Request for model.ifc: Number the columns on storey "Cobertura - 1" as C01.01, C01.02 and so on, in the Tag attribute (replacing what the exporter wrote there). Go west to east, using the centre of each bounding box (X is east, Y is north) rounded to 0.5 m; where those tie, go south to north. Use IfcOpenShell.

First a look at what the model holds.

```python
import ifcopenshell
import ifcopenshell.util.element
import ifcopenshell.util.placement

model = ifcopenshell.open("model.ifc")
print(model.schema)
storey = next(s for s in model.by_type("IfcBuildingStorey") if s.Name == "Cobertura - 1")
columns = [e for e in ifcopenshell.util.element.get_decomposition(storey) if e.is_a("IfcColumn")]
for e in sorted(columns, key=lambda e: e.id()):
    origin = ifcopenshell.util.placement.get_local_placement(e.ObjectPlacement)[:3, 3]
    print(e.id(), e.Tag, e.Name, origin.round(2) + 0.0, sep=" | ")
```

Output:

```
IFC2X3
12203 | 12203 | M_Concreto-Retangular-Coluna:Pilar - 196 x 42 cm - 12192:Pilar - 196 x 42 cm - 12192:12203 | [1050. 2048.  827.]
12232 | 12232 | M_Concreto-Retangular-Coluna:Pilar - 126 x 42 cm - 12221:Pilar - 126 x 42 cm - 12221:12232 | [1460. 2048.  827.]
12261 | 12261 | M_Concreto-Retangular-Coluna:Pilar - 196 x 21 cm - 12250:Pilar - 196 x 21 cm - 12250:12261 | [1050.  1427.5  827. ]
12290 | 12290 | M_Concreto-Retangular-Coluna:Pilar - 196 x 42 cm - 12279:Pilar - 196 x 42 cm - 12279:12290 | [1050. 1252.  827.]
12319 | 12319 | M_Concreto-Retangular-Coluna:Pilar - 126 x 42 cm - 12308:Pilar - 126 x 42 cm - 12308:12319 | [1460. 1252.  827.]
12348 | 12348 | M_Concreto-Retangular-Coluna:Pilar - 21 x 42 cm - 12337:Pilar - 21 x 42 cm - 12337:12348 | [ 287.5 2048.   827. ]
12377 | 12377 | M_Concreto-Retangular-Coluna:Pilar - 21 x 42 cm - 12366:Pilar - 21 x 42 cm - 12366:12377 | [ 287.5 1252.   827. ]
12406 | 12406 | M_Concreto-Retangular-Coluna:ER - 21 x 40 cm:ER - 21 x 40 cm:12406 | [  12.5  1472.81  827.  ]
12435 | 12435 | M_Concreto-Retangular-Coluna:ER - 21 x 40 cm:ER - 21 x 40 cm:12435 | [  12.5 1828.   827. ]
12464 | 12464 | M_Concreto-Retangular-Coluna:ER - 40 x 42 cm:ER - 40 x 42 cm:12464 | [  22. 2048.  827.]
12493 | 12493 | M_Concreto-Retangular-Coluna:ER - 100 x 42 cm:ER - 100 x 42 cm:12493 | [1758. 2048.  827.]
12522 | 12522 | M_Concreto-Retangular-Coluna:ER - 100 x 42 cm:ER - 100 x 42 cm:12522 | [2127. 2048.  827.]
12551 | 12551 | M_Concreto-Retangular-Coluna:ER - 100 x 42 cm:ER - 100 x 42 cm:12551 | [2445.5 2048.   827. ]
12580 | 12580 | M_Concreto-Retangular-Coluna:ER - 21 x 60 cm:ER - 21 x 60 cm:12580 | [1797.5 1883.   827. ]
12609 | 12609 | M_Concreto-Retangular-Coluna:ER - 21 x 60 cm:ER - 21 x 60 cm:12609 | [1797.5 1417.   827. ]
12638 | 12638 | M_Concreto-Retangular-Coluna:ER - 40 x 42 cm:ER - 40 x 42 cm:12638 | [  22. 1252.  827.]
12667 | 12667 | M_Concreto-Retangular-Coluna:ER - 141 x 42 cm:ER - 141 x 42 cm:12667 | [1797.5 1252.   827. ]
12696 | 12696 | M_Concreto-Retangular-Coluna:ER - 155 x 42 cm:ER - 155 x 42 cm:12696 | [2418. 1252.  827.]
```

```python
import ifcopenshell
import ifcopenshell.geom
import ifcopenshell.util.element
import ifcopenshell.util.shape

model = ifcopenshell.open("model.ifc")
settings = ifcopenshell.geom.settings()
settings.set("use-world-coords", True)


def centre(element):
    shape = ifcopenshell.geom.create_shape(settings, element)
    return ifcopenshell.util.shape.get_bbox_centroid(shape.geometry)


storey = next(s for s in model.by_type("IfcBuildingStorey") if s.Name == "Cobertura - 1")
columns = [e for e in ifcopenshell.util.element.get_decomposition(storey) if e.is_a("IfcColumn")]

# Insertion points can sit at a corner or the storey origin, so sort by the geometry (in metres).
centres = {e: centre(e) for e in columns}
columns.sort(key=lambda e: (round(centres[e][0] / 0.5), centres[e][1]))

for i, e in enumerate(columns, start=1):
    number = f"C01.{i:02d}"
    e.Tag = number
    print(e.id(), number)

model.write("model_updated.ifc")
```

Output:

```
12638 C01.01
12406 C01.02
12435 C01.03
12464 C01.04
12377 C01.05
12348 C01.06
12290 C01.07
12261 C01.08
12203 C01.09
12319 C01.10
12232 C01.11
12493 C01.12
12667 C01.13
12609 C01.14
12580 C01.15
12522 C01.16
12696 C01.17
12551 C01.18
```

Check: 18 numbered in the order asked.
